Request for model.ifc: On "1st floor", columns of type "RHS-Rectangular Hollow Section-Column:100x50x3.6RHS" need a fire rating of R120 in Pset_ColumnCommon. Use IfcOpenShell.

First a look at what the model holds.

```python
import ifcopenshell
import ifcopenshell.util.element

model = ifcopenshell.open("model.ifc")
print(model.schema)
storey = next(s for s in model.by_type("IfcBuildingStorey") if s.Name == "1st floor")
columns = [e for e in ifcopenshell.util.element.get_decomposition(storey) if e.is_a("IfcColumn")]
seen = {}
for e in columns:
    element_type = ifcopenshell.util.element.get_type(e)
    key = (element_type.Name if element_type != e and element_type else None, ifcopenshell.util.element.get_pset(e, "Pset_ColumnCommon", "FireRating"))
    seen[key] = seen.get(key, 0) + 1
for (name, value), count in sorted(seen.items(), key=str):
    print(count, "x", name, "|", value)
```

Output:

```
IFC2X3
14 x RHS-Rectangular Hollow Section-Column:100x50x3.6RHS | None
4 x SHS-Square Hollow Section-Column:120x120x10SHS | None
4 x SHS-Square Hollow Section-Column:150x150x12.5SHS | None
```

```python
import ifcopenshell
import ifcopenshell.api.pset
import ifcopenshell.util.element

model = ifcopenshell.open("model.ifc")

storey = next(s for s in model.by_type("IfcBuildingStorey") if s.Name == "1st floor")
columns = [e for e in ifcopenshell.util.element.get_decomposition(storey) if e.is_a("IfcColumn")]

count = 0
for e in columns:
    element_type = ifcopenshell.util.element.get_type(e)
    if element_type in (None, e) or element_type.Name != "RHS-Rectangular Hollow Section-Column:100x50x3.6RHS":
        continue
    # add_pset returns the element's existing set when there is one.
    pset = ifcopenshell.api.pset.add_pset(model, product=e, name="Pset_ColumnCommon")
    ifcopenshell.api.pset.edit_pset(model, pset=pset, properties={"FireRating": "R120"})
    count += 1

print(count, "columns updated")

model.write("model_v2.ifc")
```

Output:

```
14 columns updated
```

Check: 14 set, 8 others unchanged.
